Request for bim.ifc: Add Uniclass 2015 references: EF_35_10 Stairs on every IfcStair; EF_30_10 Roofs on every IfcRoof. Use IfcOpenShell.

First a look at what the model holds.

```python
import ifcopenshell

model = ifcopenshell.open("bim.ifc")
print(model.schema)
print("classifications:", [c.Name for c in model.by_type("IfcClassification")])
for ifc_class in ("IfcDoor", "IfcRoof", "IfcStair", "IfcWall", "IfcWindow"):
    print(ifc_class, len(model.by_type(ifc_class)))
```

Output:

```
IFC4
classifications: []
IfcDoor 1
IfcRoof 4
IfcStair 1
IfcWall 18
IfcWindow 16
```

```python
import ifcopenshell
import ifcopenshell.api.classification

model = ifcopenshell.open("bim.ifc")

system = ifcopenshell.api.classification.add_classification(model, classification="Uniclass 2015")

codes = {
    "IfcStair": ("EF_35_10", "Stairs"),
    "IfcRoof": ("EF_30_10", "Roofs"),
}
for ifc_class, (code, name) in codes.items():
    products = model.by_type(ifc_class)
    ifcopenshell.api.classification.add_reference(
        model, products=products, classification=system, identification=code, name=name
    )
    print(code, len(products))

model.write("bim_rev.ifc")
```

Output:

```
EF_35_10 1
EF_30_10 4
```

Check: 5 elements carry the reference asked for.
